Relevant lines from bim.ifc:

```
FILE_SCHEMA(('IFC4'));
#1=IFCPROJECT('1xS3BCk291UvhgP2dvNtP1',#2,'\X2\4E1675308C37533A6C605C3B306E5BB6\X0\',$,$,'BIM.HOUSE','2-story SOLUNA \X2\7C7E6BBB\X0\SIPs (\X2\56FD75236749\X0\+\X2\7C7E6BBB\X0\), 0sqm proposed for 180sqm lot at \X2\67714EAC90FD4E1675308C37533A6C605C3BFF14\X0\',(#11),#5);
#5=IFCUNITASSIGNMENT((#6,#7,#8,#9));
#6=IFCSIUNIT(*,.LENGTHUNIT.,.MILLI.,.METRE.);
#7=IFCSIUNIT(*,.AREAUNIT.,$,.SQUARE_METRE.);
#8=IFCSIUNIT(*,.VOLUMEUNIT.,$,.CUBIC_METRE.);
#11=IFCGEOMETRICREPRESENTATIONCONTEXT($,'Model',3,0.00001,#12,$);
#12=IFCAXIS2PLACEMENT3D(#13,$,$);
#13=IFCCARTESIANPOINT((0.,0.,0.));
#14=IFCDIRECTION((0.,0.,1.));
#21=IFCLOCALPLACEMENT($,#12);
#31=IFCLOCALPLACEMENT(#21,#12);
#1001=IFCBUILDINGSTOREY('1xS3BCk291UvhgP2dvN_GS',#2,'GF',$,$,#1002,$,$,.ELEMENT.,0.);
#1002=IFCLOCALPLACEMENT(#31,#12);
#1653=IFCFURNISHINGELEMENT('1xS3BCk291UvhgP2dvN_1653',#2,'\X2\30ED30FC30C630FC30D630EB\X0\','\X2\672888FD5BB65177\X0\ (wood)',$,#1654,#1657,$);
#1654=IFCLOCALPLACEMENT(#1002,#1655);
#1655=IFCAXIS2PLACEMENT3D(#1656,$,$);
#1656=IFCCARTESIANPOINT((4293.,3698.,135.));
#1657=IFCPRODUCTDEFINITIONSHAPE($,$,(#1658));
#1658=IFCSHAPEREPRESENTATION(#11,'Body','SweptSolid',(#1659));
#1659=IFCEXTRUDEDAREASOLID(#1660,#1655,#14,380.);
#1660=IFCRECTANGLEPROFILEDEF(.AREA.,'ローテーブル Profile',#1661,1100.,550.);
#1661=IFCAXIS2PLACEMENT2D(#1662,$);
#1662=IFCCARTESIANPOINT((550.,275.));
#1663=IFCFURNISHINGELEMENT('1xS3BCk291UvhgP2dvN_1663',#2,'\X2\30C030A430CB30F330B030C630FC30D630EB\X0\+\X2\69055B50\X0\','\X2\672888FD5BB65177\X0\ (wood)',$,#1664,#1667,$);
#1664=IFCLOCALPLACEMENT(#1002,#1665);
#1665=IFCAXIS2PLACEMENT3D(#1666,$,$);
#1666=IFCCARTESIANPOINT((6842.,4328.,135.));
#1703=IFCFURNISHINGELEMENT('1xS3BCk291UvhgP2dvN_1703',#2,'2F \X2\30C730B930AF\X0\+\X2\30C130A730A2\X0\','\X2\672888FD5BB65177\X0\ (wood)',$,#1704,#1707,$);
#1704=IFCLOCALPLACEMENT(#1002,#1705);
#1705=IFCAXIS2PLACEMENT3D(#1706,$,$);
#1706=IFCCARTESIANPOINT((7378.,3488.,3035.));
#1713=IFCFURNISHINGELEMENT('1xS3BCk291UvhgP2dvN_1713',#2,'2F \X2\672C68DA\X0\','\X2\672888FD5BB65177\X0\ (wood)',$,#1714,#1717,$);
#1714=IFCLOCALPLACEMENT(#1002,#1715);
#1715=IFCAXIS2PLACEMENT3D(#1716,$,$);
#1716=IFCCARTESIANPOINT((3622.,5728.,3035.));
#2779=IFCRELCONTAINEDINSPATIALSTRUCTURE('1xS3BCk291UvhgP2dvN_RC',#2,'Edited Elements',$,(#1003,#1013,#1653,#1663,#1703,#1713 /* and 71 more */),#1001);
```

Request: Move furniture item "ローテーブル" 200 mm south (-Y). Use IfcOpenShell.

```python
import ifcopenshell
import ifcopenshell.api.geometry
import ifcopenshell.util.placement

model = ifcopenshell.open("bim.ifc")

item = model.by_id(1653)
matrix = ifcopenshell.util.placement.get_local_placement(item.ObjectPlacement)
matrix[1, 3] -= 200.0
ifcopenshell.api.geometry.edit_object_placement(model, product=item, matrix=matrix, is_si=False)

print(ifcopenshell.util.placement.get_local_placement(item.ObjectPlacement).round(3) + 0.0)

model.write("bim-out.ifc")
```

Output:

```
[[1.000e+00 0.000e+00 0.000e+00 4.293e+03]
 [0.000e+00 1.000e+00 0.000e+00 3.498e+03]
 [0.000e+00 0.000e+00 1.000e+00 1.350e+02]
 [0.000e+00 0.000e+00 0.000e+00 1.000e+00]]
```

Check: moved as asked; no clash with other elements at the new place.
